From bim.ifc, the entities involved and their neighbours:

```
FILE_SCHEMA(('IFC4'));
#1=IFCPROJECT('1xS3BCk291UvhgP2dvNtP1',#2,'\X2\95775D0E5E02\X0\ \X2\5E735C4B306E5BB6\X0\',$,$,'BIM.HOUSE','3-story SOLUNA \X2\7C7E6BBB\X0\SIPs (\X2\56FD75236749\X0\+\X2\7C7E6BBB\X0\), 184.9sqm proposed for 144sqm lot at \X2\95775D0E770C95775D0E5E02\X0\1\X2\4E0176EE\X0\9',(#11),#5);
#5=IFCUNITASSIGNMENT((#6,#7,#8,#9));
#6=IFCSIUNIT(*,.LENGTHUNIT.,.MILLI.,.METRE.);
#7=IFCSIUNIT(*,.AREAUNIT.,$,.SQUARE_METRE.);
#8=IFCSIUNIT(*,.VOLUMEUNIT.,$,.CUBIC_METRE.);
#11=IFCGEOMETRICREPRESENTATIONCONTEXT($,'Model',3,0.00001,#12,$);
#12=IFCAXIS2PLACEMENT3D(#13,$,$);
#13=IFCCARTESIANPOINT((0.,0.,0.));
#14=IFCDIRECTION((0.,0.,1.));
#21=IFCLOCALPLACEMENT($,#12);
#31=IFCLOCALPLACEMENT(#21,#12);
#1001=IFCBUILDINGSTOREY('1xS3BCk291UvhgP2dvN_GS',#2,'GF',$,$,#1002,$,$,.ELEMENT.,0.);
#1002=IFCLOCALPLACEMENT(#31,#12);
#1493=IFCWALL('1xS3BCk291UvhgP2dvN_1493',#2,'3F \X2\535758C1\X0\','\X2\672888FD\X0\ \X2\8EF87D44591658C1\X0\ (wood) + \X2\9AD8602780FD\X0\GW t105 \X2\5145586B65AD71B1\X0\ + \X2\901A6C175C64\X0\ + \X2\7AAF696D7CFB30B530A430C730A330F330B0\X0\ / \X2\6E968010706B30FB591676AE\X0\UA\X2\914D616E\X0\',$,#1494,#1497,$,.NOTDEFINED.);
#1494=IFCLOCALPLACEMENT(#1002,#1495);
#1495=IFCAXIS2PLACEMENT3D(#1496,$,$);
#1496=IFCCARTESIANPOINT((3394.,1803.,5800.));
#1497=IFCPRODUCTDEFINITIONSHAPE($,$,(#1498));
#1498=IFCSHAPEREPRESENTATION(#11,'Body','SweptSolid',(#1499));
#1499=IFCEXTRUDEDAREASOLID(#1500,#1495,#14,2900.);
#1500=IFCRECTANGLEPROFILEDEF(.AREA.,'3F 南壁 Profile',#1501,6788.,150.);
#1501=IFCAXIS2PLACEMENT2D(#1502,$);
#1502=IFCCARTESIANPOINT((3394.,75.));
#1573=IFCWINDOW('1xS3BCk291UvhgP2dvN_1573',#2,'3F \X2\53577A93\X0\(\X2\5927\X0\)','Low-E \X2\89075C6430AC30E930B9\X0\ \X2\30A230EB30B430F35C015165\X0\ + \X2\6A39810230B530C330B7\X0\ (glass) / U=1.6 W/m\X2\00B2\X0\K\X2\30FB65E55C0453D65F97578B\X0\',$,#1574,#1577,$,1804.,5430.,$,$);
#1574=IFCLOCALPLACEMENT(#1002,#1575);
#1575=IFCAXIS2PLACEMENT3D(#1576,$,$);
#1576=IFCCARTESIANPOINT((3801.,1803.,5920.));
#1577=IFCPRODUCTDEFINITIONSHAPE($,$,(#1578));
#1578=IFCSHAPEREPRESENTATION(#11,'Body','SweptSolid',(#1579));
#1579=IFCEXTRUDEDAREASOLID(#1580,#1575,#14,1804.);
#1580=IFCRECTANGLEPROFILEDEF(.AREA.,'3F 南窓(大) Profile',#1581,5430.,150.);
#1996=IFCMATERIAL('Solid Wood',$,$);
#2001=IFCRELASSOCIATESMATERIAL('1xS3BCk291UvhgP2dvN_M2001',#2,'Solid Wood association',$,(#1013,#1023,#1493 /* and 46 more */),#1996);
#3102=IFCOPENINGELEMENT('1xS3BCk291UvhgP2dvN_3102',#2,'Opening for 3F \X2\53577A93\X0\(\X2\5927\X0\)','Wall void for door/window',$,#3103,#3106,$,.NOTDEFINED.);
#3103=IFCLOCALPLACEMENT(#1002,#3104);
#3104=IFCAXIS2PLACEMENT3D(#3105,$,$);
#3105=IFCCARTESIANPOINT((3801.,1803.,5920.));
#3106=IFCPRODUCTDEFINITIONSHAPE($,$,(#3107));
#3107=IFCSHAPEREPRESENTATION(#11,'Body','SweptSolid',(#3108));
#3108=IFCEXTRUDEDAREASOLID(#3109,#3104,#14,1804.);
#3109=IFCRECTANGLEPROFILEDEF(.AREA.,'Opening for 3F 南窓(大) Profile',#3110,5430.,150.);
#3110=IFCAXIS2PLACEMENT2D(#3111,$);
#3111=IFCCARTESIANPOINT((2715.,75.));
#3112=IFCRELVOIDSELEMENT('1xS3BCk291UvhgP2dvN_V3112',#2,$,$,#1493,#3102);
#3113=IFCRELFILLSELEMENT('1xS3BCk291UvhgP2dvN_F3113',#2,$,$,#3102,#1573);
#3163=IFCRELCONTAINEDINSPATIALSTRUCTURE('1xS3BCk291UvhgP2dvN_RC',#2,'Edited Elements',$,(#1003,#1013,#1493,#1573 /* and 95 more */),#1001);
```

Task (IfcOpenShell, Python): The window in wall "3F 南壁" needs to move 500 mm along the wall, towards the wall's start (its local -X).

```python
import ifcopenshell
import ifcopenshell.api.geometry
import ifcopenshell.util.placement
import ifcopenshell.util.unit

model = ifcopenshell.open("bim.ifc")
unit_scale = ifcopenshell.util.unit.calculate_unit_scale(model)

window = model.by_id(1573)
opening = window.FillsVoids[0].RelatingOpeningElement
wall = opening.VoidsElements[0].RelatingBuildingElement

wall_matrix = ifcopenshell.util.placement.get_local_placement(wall.ObjectPlacement)
shift = wall_matrix[:3, 0] * -0.5 / unit_scale
before = ifcopenshell.util.placement.get_local_placement(window.ObjectPlacement)[:3, 3].copy()

# The window is not placed relative to its opening, so move both.
for product in (opening, window):
    matrix = ifcopenshell.util.placement.get_local_placement(product.ObjectPlacement)
    matrix[:3, 3] += shift
    ifcopenshell.api.geometry.edit_object_placement(model, product=product, matrix=matrix, is_si=False)

after = ifcopenshell.util.placement.get_local_placement(window.ObjectPlacement)[:3, 3]
print("window moved by", (after - before).round(3) + 0.0)

model.write("bim_edited.ifc")
```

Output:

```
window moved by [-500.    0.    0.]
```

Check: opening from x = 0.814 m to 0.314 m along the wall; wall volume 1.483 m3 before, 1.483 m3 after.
